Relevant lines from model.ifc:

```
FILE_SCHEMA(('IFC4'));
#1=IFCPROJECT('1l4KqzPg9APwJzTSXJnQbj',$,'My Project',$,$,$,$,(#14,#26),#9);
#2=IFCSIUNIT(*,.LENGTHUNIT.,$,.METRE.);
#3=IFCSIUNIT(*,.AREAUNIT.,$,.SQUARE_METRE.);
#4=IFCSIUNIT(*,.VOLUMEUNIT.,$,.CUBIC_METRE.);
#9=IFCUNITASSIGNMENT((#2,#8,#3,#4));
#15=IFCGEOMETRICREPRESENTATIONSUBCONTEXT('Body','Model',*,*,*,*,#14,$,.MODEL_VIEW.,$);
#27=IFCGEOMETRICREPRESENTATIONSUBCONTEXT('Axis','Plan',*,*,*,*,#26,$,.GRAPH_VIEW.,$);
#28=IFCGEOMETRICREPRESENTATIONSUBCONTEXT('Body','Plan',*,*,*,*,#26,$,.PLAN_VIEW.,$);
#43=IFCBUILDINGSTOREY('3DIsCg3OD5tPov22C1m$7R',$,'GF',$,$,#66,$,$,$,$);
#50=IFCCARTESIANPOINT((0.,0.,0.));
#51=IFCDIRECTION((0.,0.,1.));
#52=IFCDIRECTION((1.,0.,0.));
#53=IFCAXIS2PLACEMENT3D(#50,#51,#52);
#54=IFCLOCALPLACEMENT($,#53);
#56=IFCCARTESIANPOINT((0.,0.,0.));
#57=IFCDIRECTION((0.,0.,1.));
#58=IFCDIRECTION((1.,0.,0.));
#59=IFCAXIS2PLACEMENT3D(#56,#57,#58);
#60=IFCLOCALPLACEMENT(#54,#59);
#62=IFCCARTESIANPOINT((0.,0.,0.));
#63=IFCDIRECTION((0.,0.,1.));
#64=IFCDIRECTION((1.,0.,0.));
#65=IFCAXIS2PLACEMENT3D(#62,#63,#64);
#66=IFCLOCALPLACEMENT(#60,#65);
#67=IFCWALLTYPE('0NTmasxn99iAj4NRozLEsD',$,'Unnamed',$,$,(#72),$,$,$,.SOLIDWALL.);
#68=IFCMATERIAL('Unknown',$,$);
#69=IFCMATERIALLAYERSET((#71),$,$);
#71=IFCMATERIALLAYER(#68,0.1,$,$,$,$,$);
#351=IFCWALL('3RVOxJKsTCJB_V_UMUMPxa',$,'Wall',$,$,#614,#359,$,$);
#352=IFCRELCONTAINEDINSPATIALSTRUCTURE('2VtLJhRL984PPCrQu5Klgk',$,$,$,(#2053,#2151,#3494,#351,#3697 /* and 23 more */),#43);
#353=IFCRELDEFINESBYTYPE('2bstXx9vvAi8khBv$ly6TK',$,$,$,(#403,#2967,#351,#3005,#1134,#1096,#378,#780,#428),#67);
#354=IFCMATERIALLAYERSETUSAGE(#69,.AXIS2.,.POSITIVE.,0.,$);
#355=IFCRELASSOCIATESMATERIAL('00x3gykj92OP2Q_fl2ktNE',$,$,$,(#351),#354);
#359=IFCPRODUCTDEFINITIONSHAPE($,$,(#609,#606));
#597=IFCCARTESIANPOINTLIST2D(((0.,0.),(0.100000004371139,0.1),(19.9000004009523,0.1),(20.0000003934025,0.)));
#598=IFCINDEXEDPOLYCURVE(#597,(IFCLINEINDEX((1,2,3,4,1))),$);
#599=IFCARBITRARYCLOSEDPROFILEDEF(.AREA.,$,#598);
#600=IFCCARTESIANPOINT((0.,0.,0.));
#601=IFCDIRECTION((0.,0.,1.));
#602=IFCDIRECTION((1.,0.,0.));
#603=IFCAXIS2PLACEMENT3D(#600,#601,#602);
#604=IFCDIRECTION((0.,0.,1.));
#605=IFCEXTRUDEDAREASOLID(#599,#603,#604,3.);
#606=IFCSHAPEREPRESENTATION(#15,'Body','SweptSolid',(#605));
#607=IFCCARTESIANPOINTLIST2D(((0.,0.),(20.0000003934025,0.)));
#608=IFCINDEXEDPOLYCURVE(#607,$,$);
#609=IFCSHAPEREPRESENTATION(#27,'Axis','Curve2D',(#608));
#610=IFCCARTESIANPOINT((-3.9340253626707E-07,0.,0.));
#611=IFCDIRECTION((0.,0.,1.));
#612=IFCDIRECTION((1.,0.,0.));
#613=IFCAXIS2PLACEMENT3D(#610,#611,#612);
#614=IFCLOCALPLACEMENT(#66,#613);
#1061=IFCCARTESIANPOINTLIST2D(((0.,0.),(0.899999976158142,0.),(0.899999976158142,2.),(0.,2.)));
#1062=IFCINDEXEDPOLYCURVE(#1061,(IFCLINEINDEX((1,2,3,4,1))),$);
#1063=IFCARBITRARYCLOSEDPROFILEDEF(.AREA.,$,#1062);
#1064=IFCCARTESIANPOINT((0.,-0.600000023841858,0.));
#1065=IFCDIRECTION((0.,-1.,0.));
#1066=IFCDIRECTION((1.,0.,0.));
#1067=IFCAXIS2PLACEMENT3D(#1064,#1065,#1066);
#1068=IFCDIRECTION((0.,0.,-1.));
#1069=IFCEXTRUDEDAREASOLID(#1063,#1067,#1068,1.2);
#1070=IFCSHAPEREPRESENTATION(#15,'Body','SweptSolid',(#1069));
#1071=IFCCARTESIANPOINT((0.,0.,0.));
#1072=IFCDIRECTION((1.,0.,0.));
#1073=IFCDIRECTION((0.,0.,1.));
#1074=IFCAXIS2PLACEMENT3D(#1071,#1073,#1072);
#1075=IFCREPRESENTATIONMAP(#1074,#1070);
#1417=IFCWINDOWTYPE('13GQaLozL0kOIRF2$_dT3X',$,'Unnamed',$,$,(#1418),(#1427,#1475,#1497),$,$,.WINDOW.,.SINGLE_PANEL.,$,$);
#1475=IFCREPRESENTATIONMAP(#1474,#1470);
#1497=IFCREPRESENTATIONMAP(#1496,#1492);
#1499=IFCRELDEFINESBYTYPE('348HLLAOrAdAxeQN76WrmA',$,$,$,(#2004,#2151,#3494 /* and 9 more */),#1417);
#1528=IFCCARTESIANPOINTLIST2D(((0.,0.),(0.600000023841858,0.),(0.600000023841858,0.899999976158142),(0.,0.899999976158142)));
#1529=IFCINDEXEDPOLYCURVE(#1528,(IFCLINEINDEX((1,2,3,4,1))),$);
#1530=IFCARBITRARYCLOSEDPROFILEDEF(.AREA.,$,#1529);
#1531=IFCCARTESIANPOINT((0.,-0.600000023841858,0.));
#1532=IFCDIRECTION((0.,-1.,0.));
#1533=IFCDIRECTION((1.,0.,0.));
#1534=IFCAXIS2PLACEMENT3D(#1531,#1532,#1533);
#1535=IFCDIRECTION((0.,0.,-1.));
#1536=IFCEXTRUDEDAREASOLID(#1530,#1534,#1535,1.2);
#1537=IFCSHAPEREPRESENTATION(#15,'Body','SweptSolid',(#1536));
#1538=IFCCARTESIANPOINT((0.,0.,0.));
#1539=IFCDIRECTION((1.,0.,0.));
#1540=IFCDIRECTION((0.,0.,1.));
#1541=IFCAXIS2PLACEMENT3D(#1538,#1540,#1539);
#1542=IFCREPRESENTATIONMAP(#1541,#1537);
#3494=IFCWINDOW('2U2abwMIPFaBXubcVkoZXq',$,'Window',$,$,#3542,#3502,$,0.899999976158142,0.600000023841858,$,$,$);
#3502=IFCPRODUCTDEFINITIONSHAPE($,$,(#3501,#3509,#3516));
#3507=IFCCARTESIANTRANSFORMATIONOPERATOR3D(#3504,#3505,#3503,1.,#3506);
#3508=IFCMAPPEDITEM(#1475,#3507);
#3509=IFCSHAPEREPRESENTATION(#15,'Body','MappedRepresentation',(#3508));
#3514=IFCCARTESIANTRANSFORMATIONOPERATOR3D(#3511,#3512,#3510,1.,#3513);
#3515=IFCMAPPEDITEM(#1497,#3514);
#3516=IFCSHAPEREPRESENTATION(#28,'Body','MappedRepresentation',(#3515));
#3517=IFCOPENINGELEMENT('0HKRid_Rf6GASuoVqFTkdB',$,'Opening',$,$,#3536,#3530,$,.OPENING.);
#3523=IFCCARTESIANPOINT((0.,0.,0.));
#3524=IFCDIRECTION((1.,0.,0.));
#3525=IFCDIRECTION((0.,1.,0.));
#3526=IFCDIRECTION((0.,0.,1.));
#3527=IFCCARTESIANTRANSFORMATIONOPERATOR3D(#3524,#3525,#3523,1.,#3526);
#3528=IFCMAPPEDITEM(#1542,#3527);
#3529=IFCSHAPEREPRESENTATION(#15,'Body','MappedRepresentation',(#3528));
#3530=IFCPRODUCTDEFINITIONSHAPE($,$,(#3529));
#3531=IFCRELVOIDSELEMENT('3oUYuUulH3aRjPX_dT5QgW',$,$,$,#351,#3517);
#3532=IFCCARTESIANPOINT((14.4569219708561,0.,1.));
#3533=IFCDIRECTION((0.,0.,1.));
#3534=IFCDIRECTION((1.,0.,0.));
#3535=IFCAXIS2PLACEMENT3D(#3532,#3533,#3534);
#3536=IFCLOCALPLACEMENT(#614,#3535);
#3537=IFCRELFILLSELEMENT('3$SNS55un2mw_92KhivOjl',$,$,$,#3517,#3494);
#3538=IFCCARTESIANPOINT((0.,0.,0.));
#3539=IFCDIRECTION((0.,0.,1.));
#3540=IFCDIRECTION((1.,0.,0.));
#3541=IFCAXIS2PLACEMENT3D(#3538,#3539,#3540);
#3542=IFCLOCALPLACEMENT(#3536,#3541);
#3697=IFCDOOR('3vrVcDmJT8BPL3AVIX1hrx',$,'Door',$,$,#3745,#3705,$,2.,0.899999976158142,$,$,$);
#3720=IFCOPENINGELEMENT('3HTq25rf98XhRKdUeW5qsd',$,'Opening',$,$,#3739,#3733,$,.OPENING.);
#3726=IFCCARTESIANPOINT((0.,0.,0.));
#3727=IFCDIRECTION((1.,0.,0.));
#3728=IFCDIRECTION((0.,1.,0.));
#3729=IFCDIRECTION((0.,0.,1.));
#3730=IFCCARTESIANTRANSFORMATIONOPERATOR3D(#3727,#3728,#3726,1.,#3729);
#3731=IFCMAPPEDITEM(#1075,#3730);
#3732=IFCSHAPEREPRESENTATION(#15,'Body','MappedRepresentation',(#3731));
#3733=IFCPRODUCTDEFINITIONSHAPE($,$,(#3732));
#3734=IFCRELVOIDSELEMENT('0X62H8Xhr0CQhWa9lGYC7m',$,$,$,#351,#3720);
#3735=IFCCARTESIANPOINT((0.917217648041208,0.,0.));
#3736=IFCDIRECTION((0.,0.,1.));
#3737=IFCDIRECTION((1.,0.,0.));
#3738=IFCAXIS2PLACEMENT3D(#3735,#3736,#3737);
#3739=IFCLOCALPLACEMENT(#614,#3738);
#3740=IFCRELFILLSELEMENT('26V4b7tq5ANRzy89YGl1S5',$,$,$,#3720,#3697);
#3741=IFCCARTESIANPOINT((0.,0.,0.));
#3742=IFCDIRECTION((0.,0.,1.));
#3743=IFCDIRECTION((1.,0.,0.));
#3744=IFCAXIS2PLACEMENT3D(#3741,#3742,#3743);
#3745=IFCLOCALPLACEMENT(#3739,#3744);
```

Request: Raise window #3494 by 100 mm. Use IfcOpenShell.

```python
import numpy as np
import ifcopenshell
import ifcopenshell.api.geometry
import ifcopenshell.util.placement
import ifcopenshell.util.unit

model = ifcopenshell.open("model.ifc")
unit_scale = ifcopenshell.util.unit.calculate_unit_scale(model)

window = model.by_id(3494)
opening = window.FillsVoids[0].RelatingOpeningElement
dz = 0.1 / unit_scale

shift = np.array([0.0, 0.0, dz])
# The window is placed relative to its opening, so it follows when the opening moves.
matrix = ifcopenshell.util.placement.get_local_placement(opening.ObjectPlacement)
matrix[:3, 3] += shift
ifcopenshell.api.geometry.edit_object_placement(
    model, product=opening, matrix=matrix, is_si=False, should_transform_children=True
)

print(f"moved by {dz * unit_scale:+.3f} m")

model.write("model_updated.ifc")
```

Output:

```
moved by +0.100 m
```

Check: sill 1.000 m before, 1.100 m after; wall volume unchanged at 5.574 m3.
